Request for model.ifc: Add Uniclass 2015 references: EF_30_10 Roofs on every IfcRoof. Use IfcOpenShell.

First a look at what the model holds.

```python
import ifcopenshell

model = ifcopenshell.open("model.ifc")
print(model.schema)
print("classifications:", [c.Name for c in model.by_type("IfcClassification")])
for ifc_class in ("IfcDoor", "IfcRoof", "IfcStair", "IfcWall", "IfcWindow"):
    print(ifc_class, len(model.by_type(ifc_class)))
```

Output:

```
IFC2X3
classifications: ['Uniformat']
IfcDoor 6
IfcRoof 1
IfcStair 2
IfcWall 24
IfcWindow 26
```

```python
import ifcopenshell
import ifcopenshell.api.classification

model = ifcopenshell.open("model.ifc")

# IFC2X3 requires Source and Edition and has no link from the project to the system.
system = model.create_entity("IfcClassification", Source="NBS", Edition="2015", Name="Uniclass 2015")

codes = {
    "IfcRoof": ("EF_30_10", "Roofs"),
}
for ifc_class, (code, name) in codes.items():
    products = model.by_type(ifc_class)
    ifcopenshell.api.classification.add_reference(
        model, products=products, classification=system, identification=code, name=name
    )
    print(code, len(products))

model.write("model_edited.ifc")
```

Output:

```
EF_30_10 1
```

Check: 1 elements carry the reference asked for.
